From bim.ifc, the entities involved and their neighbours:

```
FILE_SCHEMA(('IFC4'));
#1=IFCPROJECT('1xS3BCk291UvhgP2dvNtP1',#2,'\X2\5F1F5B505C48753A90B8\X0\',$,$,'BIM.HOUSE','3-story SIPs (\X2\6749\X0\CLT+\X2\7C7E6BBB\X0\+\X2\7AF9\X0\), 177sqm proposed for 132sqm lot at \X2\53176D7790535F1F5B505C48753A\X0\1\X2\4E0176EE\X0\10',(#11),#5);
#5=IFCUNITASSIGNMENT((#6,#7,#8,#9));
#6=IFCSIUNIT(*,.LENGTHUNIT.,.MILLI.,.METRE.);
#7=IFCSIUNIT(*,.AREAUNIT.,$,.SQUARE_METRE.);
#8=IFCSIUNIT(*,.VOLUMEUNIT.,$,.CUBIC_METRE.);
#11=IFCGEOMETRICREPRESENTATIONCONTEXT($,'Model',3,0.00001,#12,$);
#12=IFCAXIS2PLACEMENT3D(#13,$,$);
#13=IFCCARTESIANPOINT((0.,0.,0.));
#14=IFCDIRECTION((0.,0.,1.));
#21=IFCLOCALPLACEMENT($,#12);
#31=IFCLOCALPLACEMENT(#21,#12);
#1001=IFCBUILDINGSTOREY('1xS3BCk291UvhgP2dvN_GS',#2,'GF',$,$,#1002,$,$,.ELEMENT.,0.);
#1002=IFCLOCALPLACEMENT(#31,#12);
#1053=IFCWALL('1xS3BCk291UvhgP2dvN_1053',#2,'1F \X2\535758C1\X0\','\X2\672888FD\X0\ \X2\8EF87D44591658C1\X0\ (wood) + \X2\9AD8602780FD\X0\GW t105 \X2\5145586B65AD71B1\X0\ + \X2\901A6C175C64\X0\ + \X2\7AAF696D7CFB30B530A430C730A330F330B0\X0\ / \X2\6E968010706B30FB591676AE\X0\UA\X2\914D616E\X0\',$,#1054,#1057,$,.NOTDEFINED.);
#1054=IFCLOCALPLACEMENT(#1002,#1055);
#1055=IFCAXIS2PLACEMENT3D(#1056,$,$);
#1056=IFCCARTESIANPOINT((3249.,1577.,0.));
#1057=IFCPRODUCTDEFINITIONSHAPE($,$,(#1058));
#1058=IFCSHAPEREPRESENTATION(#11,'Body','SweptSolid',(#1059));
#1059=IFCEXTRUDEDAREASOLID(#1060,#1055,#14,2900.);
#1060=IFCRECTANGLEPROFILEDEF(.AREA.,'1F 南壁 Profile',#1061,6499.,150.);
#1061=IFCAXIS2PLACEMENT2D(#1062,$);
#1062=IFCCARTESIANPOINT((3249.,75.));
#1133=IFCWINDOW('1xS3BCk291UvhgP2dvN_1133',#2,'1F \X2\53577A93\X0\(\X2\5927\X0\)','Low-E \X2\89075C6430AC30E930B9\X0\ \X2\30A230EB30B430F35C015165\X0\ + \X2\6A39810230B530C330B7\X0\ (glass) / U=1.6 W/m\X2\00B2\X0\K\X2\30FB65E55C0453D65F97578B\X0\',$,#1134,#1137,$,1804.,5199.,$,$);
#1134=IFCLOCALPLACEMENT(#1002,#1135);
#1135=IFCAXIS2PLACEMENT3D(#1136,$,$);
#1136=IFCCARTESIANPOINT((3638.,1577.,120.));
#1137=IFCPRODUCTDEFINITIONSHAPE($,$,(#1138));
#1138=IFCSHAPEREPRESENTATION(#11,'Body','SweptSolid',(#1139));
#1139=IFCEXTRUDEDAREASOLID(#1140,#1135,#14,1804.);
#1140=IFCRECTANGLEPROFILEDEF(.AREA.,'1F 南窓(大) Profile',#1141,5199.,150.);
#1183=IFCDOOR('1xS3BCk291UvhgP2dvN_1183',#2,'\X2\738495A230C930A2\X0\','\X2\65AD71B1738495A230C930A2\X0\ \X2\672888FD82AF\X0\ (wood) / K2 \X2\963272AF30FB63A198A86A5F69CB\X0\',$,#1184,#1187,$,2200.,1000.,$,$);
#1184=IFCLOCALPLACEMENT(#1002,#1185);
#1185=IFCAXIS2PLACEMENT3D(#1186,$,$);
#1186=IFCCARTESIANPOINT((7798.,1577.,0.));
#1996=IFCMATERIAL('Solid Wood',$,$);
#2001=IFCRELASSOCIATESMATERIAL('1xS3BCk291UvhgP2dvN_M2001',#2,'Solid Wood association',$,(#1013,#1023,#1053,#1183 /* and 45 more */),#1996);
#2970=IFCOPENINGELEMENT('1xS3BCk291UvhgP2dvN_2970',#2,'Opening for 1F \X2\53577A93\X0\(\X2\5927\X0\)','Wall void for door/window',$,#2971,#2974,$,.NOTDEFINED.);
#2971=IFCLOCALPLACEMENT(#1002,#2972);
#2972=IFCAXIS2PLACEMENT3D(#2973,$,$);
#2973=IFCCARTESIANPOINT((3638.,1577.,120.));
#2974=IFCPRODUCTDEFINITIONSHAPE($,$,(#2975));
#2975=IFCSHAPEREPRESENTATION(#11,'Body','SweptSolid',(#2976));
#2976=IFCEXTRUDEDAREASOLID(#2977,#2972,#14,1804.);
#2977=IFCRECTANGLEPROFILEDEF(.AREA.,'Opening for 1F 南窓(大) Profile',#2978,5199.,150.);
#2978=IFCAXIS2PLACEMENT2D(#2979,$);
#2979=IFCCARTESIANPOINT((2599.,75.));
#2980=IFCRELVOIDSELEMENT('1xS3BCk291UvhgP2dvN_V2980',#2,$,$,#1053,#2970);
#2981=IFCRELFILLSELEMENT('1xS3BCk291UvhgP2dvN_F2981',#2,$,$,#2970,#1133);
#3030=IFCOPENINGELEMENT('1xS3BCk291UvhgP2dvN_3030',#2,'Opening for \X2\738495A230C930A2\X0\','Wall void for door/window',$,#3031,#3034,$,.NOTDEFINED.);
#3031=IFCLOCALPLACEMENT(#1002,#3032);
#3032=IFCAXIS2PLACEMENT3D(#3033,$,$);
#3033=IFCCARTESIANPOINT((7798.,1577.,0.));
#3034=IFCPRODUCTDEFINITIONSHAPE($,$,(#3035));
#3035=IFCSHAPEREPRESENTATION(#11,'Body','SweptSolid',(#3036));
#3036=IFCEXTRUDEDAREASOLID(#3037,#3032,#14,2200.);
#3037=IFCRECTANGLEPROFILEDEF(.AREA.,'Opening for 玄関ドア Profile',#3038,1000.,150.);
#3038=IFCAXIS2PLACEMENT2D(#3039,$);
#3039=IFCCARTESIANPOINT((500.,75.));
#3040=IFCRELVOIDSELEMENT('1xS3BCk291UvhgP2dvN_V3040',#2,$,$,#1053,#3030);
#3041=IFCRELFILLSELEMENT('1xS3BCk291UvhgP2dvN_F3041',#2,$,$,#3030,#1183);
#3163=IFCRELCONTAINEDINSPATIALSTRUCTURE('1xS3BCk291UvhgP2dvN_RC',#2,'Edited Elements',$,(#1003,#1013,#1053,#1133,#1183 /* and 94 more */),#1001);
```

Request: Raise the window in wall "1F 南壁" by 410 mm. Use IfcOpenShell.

```python
import numpy as np
import ifcopenshell
import ifcopenshell.api.geometry
import ifcopenshell.util.placement
import ifcopenshell.util.unit

model = ifcopenshell.open("bim.ifc")
unit_scale = ifcopenshell.util.unit.calculate_unit_scale(model)

window = model.by_id(1133)
opening = window.FillsVoids[0].RelatingOpeningElement
dz = 0.41 / unit_scale

shift = np.array([0.0, 0.0, dz])
# The window is not placed relative to its opening, so move both.
for product in (opening, window):
    matrix = ifcopenshell.util.placement.get_local_placement(product.ObjectPlacement)
    matrix[:3, 3] += shift
    ifcopenshell.api.geometry.edit_object_placement(model, product=product, matrix=matrix, is_si=False)

print(f"moved by {dz * unit_scale:+.3f} m")

model.write("bim_rev.ifc")
```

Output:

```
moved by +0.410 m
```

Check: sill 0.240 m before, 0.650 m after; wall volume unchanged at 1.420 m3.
